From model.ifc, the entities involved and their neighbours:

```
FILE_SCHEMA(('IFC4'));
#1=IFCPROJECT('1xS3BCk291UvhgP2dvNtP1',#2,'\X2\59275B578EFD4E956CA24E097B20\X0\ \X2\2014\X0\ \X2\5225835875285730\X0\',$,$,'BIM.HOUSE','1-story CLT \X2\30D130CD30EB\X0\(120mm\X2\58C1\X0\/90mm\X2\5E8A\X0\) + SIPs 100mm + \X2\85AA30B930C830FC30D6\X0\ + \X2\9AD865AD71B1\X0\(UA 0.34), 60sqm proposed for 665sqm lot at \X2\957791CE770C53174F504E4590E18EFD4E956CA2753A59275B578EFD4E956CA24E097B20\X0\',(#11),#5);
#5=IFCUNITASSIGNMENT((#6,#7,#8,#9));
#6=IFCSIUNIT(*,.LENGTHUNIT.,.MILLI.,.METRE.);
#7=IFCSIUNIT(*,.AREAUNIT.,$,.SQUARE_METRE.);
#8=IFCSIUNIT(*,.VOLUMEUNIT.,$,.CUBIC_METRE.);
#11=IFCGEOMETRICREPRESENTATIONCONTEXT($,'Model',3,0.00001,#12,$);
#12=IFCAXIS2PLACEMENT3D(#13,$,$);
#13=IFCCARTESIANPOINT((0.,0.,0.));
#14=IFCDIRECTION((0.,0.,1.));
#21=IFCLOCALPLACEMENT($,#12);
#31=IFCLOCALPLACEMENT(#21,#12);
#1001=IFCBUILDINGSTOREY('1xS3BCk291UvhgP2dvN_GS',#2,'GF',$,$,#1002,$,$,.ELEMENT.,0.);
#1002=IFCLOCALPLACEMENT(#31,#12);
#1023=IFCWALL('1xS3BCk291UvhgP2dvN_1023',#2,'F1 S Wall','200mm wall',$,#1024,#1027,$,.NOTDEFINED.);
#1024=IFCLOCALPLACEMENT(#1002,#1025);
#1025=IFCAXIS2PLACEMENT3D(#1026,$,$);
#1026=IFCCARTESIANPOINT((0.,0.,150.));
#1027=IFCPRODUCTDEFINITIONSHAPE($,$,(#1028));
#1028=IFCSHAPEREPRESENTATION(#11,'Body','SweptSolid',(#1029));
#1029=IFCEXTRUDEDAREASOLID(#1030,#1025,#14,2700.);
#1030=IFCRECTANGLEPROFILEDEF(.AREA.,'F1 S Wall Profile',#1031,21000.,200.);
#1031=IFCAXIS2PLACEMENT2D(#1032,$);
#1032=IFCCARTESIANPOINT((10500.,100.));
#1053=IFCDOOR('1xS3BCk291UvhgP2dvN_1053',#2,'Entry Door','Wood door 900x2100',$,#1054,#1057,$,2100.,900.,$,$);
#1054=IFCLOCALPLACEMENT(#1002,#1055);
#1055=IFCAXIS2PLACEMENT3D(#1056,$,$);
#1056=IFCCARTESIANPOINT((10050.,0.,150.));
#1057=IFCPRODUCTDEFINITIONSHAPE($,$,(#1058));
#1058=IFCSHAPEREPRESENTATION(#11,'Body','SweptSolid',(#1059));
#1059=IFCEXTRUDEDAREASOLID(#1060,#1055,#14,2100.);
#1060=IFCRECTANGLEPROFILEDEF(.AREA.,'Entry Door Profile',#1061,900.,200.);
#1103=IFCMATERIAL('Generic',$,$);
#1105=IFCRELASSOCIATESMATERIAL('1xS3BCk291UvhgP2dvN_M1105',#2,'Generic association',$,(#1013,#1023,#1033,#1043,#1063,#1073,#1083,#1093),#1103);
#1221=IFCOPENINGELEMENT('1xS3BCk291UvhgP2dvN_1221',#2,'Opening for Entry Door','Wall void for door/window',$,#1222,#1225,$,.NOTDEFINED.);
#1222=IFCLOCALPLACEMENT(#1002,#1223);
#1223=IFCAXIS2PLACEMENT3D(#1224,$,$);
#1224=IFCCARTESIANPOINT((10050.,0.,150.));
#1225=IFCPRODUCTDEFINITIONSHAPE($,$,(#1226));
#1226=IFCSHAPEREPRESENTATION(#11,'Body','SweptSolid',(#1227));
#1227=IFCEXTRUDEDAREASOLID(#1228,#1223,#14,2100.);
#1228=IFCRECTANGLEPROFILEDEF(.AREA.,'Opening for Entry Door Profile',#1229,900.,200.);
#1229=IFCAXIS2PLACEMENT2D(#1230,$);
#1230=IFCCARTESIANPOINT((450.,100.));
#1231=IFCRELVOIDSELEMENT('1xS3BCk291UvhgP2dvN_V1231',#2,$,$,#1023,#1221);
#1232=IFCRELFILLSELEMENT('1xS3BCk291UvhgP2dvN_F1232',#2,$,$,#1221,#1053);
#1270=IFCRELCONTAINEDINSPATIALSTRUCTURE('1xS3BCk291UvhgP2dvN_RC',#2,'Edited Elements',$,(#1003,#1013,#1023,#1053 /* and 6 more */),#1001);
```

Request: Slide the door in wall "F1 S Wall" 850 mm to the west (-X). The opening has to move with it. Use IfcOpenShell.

```python
import ifcopenshell
import ifcopenshell.api.geometry
import ifcopenshell.util.placement

model = ifcopenshell.open("model.ifc")

door = model.by_guid("1xS3BCk291UvhgP2dvN_1053")
opening = door.FillsVoids[0].RelatingOpeningElement
wall = opening.VoidsElements[0].RelatingBuildingElement

wall_matrix = ifcopenshell.util.placement.get_local_placement(wall.ObjectPlacement)
shift = wall_matrix[:3, 0] * -850.0
before = ifcopenshell.util.placement.get_local_placement(door.ObjectPlacement)[:3, 3].copy()

# The door is not placed relative to its opening, so move both.
for product in (opening, door):
    matrix = ifcopenshell.util.placement.get_local_placement(product.ObjectPlacement)
    matrix[:3, 3] += shift
    ifcopenshell.api.geometry.edit_object_placement(model, product=product, matrix=matrix, is_si=False)

after = ifcopenshell.util.placement.get_local_placement(door.ObjectPlacement)[:3, 3]
print("door moved by", (after - before).round(3) + 0.0)

model.write("model_edited.ifc")
```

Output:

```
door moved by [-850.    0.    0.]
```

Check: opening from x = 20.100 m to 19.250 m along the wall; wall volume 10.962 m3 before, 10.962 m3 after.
